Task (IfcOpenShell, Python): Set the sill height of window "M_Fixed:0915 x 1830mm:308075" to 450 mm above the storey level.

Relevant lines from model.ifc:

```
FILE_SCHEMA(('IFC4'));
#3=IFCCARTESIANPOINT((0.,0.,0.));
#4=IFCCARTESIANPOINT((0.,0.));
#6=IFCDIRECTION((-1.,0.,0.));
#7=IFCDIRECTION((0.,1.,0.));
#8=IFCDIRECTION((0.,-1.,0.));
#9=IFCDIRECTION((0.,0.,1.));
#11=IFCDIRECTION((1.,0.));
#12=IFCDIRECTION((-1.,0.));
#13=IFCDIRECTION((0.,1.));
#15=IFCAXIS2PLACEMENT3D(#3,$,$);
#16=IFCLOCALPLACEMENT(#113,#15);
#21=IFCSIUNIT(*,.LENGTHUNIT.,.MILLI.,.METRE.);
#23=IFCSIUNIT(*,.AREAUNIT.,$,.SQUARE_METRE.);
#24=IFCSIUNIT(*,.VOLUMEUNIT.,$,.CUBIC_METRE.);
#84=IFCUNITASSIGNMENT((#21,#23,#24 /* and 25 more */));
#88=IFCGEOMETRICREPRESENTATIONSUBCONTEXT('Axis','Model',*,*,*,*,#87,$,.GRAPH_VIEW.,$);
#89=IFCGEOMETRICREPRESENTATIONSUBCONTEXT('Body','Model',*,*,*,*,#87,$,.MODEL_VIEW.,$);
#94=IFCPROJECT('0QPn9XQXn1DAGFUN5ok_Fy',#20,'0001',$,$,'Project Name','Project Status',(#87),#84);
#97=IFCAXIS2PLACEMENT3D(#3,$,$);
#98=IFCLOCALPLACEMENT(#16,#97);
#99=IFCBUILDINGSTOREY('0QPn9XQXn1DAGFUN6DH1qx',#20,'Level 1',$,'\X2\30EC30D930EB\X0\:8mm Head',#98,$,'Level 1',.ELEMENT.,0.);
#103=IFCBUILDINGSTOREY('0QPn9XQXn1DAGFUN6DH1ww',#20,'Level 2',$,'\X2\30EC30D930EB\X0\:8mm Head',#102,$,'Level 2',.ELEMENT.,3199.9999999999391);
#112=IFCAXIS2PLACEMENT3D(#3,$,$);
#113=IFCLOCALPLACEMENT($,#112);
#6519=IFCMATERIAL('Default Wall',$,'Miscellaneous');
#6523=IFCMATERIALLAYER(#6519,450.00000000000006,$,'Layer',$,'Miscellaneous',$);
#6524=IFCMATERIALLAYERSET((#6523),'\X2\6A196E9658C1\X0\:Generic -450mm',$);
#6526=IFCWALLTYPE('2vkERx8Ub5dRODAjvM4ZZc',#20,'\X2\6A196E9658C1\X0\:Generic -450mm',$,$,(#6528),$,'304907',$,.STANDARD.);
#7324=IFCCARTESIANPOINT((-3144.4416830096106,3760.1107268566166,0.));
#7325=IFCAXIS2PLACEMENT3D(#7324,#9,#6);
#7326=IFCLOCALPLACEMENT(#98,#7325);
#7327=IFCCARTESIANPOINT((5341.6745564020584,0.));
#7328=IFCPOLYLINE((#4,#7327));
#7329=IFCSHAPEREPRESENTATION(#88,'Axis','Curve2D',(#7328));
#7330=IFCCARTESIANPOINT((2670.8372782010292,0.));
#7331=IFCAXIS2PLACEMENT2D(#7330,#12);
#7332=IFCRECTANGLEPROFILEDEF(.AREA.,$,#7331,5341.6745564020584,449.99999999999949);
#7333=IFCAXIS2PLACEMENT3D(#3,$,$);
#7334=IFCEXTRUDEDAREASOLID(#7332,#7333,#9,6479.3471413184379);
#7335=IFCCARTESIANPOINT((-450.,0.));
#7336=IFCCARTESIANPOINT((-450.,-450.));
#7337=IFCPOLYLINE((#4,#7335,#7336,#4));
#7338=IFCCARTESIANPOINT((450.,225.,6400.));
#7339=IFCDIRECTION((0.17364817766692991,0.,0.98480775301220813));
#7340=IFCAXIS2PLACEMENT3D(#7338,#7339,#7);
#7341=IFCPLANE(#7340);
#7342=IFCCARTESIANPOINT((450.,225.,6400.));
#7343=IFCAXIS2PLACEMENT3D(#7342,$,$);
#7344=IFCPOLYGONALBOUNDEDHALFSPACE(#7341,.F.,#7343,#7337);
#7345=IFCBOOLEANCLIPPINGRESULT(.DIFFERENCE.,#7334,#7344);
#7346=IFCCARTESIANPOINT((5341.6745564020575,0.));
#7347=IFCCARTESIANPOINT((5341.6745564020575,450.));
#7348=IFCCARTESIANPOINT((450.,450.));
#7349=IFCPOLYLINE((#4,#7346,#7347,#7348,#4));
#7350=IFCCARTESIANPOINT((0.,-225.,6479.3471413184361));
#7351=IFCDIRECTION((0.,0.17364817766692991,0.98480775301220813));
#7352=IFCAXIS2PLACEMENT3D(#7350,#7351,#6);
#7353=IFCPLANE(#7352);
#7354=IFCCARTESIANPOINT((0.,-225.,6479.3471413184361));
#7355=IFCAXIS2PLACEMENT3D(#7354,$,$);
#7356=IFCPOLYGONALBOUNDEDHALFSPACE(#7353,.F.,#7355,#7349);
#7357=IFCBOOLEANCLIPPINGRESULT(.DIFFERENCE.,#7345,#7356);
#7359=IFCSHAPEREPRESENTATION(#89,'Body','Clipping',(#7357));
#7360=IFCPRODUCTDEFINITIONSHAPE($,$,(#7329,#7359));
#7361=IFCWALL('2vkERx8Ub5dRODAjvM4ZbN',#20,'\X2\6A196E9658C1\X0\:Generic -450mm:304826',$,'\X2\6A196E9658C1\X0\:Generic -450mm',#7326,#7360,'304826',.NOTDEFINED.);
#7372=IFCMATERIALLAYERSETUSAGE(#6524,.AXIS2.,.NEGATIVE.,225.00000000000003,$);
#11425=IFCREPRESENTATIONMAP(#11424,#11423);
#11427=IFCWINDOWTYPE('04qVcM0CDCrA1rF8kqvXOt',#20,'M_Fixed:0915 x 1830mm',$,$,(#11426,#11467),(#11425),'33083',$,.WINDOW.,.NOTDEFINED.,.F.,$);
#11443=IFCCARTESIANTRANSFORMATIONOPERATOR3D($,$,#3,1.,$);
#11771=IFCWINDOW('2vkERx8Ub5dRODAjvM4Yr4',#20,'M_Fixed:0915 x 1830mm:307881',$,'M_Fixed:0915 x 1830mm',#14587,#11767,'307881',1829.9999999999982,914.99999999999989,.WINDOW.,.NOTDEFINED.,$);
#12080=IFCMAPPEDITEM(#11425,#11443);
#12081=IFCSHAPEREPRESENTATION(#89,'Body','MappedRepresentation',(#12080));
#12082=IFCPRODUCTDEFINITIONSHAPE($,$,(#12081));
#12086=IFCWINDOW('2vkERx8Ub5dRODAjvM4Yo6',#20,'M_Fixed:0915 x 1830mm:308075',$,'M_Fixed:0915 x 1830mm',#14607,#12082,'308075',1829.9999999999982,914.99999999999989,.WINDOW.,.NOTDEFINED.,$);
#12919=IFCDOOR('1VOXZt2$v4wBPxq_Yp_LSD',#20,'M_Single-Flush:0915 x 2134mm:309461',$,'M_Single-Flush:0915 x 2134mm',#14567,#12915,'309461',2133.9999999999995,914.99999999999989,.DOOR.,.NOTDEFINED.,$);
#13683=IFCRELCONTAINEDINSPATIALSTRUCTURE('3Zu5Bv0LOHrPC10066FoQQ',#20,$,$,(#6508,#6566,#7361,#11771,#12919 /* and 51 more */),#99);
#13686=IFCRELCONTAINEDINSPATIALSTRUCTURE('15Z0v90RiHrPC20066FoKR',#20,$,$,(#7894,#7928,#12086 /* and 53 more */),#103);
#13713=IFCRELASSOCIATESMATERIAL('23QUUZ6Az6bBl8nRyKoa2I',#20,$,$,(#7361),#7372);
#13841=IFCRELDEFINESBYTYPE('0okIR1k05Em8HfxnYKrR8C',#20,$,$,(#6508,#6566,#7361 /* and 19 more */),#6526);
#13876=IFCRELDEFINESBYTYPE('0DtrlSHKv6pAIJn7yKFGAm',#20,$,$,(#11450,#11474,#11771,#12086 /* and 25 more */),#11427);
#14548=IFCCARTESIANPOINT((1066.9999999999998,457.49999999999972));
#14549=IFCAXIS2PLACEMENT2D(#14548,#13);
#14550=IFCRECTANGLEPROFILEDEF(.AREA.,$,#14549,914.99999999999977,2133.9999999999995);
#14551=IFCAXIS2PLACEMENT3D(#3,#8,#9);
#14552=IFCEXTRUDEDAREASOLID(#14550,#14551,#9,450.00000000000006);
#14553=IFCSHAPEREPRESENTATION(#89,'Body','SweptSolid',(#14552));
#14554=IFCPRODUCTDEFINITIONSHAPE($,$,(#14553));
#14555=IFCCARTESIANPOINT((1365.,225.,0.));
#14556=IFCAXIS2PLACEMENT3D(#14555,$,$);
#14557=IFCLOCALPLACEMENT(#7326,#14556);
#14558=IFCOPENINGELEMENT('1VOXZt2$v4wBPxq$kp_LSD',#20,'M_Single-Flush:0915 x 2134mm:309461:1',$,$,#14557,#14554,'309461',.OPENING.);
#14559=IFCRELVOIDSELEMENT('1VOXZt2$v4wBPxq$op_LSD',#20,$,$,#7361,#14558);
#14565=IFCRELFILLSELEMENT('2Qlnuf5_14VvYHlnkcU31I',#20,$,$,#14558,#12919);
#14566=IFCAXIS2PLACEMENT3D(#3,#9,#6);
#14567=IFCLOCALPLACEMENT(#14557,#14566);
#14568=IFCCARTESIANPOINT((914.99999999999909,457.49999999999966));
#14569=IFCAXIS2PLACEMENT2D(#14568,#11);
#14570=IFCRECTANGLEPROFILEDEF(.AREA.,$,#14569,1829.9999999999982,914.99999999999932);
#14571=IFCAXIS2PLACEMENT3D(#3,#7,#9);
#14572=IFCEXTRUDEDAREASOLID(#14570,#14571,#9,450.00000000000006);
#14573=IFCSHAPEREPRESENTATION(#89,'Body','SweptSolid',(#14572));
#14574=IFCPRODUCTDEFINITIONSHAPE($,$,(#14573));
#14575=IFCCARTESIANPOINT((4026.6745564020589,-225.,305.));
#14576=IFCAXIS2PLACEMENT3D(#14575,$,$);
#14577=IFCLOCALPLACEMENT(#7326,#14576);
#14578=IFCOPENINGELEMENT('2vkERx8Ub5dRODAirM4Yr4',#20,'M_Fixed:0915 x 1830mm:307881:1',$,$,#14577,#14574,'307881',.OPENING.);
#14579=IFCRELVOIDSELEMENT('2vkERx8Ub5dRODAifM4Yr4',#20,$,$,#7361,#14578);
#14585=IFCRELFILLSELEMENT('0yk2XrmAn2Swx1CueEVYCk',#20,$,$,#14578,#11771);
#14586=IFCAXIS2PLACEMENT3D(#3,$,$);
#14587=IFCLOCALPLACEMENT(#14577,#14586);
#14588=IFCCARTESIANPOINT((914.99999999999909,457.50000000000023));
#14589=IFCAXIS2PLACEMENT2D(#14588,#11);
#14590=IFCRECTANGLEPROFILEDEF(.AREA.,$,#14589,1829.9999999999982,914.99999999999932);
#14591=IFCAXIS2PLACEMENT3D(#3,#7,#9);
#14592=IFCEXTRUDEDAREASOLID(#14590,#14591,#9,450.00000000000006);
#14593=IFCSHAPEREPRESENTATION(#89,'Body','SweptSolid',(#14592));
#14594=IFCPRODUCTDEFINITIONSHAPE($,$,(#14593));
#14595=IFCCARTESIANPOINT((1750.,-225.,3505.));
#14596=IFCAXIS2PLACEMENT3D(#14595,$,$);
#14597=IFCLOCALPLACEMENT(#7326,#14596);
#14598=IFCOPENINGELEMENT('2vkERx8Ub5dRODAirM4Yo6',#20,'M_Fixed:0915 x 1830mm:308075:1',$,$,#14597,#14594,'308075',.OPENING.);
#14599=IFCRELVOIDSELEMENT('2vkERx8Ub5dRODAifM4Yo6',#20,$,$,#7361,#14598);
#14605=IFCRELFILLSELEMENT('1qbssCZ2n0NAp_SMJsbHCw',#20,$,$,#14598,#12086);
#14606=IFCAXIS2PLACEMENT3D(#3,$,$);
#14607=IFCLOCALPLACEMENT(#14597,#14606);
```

```python
import numpy as np
import ifcopenshell
import ifcopenshell.api.geometry
import ifcopenshell.geom
import ifcopenshell.util.element
import ifcopenshell.util.placement
import ifcopenshell.util.shape
import ifcopenshell.util.unit

model = ifcopenshell.open("model.ifc")
unit_scale = ifcopenshell.util.unit.calculate_unit_scale(model)

window = model.by_id(12086)
opening = window.FillsVoids[0].RelatingOpeningElement
storey = ifcopenshell.util.element.get_container(window, ifc_class="IfcBuildingStorey")
level = ifcopenshell.util.placement.get_local_placement(storey.ObjectPlacement)[2, 3]

# The opening's origin need not be at the sill, so measure its lowest point.
shape = ifcopenshell.geom.create_shape(ifcopenshell.geom.settings(), opening)
bottom = ifcopenshell.util.shape.get_shape_bottom_elevation(shape, shape.geometry) / unit_scale
dz = level + 450.0 - bottom

shift = np.array([0.0, 0.0, dz])
# The window is placed relative to its opening, so it follows when the opening moves.
matrix = ifcopenshell.util.placement.get_local_placement(opening.ObjectPlacement)
matrix[:3, 3] += shift
ifcopenshell.api.geometry.edit_object_placement(
    model, product=opening, matrix=matrix, is_si=False, should_transform_children=True
)

print(f"moved by {dz * unit_scale:+.3f} m")

model.write("model_rev.ifc")
```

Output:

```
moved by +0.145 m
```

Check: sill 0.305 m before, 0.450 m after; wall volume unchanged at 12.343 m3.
